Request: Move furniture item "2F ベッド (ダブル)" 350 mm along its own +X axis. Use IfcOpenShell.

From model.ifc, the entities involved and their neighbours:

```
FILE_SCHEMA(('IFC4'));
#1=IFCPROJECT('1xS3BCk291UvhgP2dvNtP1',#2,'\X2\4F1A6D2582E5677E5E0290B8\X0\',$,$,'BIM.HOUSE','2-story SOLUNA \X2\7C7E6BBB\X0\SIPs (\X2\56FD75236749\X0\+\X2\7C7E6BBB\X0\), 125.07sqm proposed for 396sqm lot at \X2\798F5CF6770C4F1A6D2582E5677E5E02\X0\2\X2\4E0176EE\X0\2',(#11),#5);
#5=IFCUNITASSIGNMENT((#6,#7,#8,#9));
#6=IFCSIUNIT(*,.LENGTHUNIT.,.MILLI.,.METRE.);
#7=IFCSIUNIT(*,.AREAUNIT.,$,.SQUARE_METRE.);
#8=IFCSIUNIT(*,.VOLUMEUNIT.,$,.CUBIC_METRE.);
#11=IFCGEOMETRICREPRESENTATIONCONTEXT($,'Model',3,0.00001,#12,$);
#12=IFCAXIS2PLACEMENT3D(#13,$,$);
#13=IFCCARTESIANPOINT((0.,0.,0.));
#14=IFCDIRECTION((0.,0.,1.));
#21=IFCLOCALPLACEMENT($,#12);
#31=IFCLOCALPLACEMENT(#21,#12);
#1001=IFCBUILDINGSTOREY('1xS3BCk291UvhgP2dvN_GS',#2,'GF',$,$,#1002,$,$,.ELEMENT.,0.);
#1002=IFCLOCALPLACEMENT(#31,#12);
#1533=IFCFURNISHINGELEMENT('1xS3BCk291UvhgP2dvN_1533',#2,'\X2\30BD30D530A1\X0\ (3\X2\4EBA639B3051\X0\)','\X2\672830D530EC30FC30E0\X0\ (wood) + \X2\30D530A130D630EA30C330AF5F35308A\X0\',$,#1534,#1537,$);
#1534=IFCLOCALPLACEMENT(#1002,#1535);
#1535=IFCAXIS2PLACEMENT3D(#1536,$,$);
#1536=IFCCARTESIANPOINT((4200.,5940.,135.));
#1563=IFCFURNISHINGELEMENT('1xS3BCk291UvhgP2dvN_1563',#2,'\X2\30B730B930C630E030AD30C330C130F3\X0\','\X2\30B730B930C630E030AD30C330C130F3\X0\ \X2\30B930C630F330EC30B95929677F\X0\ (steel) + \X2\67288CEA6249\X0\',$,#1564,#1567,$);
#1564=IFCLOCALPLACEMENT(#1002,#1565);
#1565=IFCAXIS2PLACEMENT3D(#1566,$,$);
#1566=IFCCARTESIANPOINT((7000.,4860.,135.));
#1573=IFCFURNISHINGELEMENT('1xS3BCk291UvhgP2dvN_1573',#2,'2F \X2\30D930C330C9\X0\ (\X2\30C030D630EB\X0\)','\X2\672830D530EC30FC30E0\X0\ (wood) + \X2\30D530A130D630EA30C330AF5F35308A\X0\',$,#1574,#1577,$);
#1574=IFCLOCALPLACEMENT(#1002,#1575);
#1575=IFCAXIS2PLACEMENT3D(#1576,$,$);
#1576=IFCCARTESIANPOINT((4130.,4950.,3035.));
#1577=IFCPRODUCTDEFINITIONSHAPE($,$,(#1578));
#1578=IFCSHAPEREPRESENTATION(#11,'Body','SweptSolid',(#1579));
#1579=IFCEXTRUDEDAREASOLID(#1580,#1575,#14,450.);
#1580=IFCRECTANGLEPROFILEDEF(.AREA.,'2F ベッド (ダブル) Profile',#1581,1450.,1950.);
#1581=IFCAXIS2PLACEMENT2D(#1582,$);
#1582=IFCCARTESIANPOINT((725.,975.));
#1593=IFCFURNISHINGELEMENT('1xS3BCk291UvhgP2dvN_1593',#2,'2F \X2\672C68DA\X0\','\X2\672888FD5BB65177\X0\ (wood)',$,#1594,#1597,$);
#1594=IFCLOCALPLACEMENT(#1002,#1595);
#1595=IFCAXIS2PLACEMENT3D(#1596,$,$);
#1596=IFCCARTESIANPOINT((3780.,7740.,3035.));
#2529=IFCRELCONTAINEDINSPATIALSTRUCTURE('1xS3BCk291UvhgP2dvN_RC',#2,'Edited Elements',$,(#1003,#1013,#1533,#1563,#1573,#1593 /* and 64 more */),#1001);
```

```python
import ifcopenshell
import ifcopenshell.api.geometry
import ifcopenshell.util.placement
import ifcopenshell.util.unit

model = ifcopenshell.open("model.ifc")
unit_scale = ifcopenshell.util.unit.calculate_unit_scale(model)

item = model.by_guid("1xS3BCk291UvhgP2dvN_1573")
matrix = ifcopenshell.util.placement.get_local_placement(item.ObjectPlacement)
matrix[:3, 3] += matrix[:3, 0] * 0.35 / unit_scale
ifcopenshell.api.geometry.edit_object_placement(model, product=item, matrix=matrix, is_si=False)

print(ifcopenshell.util.placement.get_local_placement(item.ObjectPlacement).round(3) + 0.0)

model.write("model_edited.ifc")
```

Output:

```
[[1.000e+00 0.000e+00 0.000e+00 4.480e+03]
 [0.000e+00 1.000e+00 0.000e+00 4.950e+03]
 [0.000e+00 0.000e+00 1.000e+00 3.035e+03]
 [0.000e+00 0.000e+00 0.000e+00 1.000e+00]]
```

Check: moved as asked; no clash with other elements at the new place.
